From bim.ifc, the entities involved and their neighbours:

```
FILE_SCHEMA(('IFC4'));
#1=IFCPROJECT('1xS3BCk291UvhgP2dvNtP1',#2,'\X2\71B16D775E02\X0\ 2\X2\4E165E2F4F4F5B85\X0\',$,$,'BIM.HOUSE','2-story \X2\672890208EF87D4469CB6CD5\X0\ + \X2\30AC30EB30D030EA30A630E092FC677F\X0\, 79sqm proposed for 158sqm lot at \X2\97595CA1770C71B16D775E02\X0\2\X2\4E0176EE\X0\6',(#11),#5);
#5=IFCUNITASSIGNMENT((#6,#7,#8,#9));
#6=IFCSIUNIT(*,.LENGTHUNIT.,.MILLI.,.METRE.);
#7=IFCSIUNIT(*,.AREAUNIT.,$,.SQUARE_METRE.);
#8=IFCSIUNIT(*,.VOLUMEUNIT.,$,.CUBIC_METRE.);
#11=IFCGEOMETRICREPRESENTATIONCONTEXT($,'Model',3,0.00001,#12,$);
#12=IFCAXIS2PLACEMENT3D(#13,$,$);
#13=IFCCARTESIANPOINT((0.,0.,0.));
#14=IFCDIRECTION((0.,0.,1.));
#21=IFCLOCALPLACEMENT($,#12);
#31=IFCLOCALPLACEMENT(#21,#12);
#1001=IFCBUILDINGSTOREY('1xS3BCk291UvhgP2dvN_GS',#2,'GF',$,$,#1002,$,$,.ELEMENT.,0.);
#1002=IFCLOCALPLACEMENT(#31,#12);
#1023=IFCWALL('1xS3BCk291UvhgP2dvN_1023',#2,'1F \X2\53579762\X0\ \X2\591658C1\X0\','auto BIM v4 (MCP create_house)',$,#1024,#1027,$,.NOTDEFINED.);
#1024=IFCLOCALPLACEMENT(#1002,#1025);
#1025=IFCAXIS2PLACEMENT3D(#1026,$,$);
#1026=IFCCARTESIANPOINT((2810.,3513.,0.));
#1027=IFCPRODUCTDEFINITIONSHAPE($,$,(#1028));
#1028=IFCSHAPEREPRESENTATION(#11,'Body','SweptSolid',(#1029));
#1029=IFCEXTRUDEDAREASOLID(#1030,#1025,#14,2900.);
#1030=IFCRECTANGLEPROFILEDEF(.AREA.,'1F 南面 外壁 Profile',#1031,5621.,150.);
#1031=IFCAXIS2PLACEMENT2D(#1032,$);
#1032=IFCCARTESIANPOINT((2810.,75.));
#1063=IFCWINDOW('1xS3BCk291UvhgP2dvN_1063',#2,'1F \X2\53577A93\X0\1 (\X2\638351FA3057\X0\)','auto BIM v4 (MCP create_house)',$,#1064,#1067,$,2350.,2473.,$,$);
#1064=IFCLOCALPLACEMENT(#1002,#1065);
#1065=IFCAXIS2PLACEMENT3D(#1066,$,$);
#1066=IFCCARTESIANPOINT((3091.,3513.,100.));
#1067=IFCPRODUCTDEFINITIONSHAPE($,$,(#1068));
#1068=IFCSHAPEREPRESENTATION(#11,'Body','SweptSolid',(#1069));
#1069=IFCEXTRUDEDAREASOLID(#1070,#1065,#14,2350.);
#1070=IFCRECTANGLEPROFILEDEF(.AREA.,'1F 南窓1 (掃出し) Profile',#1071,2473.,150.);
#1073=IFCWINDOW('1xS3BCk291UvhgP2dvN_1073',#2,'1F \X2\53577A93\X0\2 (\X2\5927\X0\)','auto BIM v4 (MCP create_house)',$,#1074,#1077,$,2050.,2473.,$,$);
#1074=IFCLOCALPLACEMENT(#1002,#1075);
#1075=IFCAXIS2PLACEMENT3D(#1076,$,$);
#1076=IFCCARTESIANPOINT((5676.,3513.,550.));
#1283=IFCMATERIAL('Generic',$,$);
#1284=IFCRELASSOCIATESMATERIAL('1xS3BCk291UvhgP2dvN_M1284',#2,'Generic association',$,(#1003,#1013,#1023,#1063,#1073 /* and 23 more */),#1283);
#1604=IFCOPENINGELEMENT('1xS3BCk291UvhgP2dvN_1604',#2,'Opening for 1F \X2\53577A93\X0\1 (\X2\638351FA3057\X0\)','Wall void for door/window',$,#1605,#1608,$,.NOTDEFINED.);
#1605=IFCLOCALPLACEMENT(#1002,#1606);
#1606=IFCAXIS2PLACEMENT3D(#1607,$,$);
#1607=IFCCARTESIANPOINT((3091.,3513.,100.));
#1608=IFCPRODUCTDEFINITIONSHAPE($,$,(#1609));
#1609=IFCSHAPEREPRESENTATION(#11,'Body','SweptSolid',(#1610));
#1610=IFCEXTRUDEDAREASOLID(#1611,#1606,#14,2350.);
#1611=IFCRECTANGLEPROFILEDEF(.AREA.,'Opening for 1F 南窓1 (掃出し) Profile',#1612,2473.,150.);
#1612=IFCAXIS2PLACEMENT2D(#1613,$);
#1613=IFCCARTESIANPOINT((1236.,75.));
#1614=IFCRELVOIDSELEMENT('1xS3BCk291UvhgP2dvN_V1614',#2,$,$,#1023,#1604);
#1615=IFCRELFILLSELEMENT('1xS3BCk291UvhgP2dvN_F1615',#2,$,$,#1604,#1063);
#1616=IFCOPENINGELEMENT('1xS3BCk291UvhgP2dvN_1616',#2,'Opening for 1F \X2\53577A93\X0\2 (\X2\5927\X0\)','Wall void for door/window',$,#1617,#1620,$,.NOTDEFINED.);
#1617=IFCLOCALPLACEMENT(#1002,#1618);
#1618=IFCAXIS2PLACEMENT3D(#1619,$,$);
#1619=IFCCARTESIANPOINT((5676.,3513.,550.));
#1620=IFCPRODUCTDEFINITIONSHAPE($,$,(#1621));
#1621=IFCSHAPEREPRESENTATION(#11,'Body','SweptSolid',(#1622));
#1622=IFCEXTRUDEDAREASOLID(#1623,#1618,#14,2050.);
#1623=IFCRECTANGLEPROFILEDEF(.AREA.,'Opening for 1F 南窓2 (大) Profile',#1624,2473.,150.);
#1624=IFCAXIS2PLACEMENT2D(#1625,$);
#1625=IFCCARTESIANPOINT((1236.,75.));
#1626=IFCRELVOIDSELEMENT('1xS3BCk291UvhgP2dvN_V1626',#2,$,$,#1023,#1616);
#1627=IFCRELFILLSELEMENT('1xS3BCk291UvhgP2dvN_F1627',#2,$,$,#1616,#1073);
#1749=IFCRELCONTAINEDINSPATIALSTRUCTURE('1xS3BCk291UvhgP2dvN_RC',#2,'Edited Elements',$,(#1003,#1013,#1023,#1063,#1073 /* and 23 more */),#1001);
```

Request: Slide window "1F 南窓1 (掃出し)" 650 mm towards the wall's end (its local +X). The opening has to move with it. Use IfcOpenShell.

```python
import ifcopenshell
import ifcopenshell.api.geometry
import ifcopenshell.util.placement
import ifcopenshell.util.unit

model = ifcopenshell.open("bim.ifc")
unit_scale = ifcopenshell.util.unit.calculate_unit_scale(model)

window = model.by_guid("1xS3BCk291UvhgP2dvN_1063")
opening = window.FillsVoids[0].RelatingOpeningElement
wall = opening.VoidsElements[0].RelatingBuildingElement

wall_matrix = ifcopenshell.util.placement.get_local_placement(wall.ObjectPlacement)
shift = wall_matrix[:3, 0] * 0.65 / unit_scale
before = ifcopenshell.util.placement.get_local_placement(window.ObjectPlacement)[:3, 3].copy()

# The window is not placed relative to its opening, so move both.
for product in (opening, window):
    matrix = ifcopenshell.util.placement.get_local_placement(product.ObjectPlacement)
    matrix[:3, 3] += shift
    ifcopenshell.api.geometry.edit_object_placement(model, product=product, matrix=matrix, is_si=False)

after = ifcopenshell.util.placement.get_local_placement(window.ObjectPlacement)[:3, 3]
print("window moved by", (after - before).round(3) + 0.0)

model.write("bim-out.ifc")
```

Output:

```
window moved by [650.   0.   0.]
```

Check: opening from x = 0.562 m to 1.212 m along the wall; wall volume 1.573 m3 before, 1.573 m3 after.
